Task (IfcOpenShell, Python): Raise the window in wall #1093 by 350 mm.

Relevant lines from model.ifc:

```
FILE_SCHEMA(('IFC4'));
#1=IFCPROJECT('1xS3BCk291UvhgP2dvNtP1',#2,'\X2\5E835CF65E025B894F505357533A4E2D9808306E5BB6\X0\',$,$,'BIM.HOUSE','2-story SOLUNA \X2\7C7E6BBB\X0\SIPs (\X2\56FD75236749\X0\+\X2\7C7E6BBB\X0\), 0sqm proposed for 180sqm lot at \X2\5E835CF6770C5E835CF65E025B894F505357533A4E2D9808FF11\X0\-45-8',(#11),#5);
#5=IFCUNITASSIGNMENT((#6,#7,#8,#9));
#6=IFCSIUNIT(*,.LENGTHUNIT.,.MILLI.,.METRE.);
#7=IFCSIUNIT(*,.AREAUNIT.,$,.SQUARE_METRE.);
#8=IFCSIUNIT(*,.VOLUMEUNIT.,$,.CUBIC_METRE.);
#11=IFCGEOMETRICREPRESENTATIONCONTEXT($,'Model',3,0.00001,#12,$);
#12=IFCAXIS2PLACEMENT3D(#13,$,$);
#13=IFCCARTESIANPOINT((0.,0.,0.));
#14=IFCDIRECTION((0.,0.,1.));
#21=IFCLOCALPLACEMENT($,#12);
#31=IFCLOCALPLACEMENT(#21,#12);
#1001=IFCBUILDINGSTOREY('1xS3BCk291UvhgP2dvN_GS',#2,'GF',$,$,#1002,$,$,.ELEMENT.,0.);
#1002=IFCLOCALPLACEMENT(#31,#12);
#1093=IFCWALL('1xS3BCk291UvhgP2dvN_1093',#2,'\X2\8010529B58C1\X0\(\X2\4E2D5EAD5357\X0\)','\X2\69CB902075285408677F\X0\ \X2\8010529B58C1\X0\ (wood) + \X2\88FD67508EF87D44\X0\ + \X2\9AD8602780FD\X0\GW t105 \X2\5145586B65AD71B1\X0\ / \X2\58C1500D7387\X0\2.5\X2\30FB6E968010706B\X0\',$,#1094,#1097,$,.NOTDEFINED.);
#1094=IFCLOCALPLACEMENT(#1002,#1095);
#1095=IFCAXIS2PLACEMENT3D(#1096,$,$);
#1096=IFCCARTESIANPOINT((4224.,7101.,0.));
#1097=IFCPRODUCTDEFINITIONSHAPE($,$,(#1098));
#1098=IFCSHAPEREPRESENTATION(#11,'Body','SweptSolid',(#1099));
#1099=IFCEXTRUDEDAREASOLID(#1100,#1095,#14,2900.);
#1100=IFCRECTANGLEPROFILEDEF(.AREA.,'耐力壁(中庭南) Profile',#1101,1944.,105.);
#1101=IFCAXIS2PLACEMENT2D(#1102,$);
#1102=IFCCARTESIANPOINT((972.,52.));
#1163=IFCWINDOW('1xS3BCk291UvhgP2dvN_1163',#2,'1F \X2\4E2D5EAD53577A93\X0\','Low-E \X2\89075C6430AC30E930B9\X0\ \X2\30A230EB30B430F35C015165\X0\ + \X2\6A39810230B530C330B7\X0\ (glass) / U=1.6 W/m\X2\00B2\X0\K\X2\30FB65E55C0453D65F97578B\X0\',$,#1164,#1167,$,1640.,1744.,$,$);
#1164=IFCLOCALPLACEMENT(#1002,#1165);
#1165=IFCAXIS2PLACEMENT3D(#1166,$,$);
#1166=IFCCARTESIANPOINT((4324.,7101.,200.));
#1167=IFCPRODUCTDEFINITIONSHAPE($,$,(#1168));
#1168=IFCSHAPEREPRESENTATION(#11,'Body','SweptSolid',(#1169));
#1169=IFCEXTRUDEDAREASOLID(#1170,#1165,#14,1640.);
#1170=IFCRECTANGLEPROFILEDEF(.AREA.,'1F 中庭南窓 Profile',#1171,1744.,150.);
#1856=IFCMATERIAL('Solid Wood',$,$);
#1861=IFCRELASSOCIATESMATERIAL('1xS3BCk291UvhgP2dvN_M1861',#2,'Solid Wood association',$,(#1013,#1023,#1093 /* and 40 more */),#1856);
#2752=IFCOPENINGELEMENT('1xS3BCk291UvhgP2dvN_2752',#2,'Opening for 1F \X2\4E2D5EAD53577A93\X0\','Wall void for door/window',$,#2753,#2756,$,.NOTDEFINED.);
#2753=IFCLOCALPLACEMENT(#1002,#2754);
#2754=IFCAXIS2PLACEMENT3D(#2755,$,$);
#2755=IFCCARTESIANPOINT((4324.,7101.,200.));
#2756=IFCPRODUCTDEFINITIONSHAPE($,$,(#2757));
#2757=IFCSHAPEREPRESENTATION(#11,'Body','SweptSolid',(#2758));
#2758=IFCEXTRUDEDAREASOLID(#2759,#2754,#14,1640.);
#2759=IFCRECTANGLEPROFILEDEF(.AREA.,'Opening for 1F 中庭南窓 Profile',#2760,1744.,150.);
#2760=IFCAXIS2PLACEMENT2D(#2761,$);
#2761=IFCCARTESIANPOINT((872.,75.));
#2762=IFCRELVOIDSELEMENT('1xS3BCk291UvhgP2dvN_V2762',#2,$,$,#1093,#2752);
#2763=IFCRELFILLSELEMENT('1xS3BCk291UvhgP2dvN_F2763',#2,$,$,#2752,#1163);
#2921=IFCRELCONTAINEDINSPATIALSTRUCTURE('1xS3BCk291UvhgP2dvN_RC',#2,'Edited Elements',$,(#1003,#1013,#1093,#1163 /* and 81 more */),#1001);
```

```python
import numpy as np
import ifcopenshell
import ifcopenshell.api.geometry
import ifcopenshell.util.placement
import ifcopenshell.util.unit

model = ifcopenshell.open("model.ifc")
unit_scale = ifcopenshell.util.unit.calculate_unit_scale(model)

window = model.by_guid("1xS3BCk291UvhgP2dvN_1163")
opening = window.FillsVoids[0].RelatingOpeningElement
dz = 350.0

shift = np.array([0.0, 0.0, dz])
# The window is not placed relative to its opening, so move both.
for product in (opening, window):
    matrix = ifcopenshell.util.placement.get_local_placement(product.ObjectPlacement)
    matrix[:3, 3] += shift
    ifcopenshell.api.geometry.edit_object_placement(model, product=product, matrix=matrix, is_si=False)

print(f"moved by {dz * unit_scale:+.3f} m")

model.write("model-out.ifc")
```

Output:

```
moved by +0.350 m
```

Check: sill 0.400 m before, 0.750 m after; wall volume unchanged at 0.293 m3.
